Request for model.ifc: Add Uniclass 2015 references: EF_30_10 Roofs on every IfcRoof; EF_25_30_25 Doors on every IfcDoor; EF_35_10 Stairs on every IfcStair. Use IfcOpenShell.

First a look at what the model holds.

```python
import ifcopenshell

model = ifcopenshell.open("model.ifc")
print(model.schema)
print("classifications:", [c.Name for c in model.by_type("IfcClassification")])
for ifc_class in ("IfcDoor", "IfcRoof", "IfcStair", "IfcWall", "IfcWindow"):
    print(ifc_class, len(model.by_type(ifc_class)))
```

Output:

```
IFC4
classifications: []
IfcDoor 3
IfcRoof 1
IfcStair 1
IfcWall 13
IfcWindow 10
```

```python
import ifcopenshell
import ifcopenshell.api.classification

model = ifcopenshell.open("model.ifc")

system = ifcopenshell.api.classification.add_classification(model, classification="Uniclass 2015")

codes = {
    "IfcRoof": ("EF_30_10", "Roofs"),
    "IfcDoor": ("EF_25_30_25", "Doors"),
    "IfcStair": ("EF_35_10", "Stairs"),
}
for ifc_class, (code, name) in codes.items():
    products = model.by_type(ifc_class)
    ifcopenshell.api.classification.add_reference(
        model, products=products, classification=system, identification=code, name=name
    )
    print(code, len(products))

model.write("model_edited.ifc")
```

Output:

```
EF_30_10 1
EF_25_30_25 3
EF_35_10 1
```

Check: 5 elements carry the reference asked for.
